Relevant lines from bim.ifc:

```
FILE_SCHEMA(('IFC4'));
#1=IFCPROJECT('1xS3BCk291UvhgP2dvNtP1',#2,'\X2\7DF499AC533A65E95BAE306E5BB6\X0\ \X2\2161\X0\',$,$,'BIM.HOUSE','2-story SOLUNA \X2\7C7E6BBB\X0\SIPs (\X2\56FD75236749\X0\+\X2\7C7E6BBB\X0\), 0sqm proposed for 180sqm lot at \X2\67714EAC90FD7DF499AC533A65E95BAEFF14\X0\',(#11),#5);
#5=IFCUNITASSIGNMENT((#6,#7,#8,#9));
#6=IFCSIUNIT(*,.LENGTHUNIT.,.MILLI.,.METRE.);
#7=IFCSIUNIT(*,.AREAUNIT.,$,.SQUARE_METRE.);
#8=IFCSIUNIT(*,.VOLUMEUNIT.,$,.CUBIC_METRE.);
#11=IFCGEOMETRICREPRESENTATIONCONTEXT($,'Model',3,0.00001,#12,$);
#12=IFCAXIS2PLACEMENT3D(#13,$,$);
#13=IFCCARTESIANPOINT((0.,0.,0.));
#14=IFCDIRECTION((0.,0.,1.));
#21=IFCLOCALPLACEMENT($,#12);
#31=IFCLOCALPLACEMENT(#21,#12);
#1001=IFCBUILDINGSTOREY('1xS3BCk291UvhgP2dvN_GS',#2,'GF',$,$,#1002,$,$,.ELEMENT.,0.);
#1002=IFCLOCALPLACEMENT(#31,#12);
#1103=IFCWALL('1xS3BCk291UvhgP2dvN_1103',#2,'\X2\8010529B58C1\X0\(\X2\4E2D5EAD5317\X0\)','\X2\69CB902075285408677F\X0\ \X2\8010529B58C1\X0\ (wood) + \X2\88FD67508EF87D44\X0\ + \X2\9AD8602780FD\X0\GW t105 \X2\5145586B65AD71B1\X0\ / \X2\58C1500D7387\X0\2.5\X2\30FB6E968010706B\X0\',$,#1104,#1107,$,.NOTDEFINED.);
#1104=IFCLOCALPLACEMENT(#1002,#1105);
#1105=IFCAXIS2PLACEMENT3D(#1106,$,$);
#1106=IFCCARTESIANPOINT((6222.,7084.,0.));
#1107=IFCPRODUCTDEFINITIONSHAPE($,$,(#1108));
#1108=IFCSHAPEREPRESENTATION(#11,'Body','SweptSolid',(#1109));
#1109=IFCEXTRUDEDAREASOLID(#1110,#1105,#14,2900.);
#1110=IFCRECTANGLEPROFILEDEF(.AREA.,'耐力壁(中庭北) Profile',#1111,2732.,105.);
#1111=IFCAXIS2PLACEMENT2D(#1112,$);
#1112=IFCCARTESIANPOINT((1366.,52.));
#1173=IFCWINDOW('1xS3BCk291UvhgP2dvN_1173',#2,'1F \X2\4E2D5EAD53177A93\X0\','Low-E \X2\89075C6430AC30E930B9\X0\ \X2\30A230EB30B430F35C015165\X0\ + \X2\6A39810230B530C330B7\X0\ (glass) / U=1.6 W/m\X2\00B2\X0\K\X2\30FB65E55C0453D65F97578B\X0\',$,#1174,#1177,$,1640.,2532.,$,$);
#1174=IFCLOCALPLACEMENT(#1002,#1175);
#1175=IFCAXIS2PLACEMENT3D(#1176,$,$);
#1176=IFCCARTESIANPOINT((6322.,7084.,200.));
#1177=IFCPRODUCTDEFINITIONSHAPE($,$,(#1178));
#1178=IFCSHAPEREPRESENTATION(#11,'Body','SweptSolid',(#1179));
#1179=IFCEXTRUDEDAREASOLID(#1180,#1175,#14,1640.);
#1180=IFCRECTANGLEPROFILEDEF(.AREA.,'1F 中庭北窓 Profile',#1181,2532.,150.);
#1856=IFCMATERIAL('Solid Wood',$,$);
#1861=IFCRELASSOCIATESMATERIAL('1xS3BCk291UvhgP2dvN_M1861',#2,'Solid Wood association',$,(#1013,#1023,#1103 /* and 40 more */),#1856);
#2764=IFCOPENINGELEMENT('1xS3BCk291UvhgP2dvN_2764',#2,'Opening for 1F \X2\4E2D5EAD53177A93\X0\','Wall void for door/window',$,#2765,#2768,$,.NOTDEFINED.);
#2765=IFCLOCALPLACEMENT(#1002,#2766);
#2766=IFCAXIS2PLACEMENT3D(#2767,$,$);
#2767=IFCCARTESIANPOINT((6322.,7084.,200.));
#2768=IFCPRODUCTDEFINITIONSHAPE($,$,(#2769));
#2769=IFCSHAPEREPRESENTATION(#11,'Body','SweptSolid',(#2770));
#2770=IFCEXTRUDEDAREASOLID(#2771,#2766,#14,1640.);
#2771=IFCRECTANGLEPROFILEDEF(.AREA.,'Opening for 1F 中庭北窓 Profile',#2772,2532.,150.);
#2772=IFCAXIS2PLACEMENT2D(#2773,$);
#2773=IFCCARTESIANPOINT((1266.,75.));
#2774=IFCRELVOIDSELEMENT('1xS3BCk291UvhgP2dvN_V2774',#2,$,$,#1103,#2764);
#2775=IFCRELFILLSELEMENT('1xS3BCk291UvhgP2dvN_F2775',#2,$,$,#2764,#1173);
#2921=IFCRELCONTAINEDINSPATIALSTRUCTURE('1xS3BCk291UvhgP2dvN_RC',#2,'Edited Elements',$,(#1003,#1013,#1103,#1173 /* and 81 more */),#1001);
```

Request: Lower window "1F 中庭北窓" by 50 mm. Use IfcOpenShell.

```python
import numpy as np
import ifcopenshell
import ifcopenshell.api.geometry
import ifcopenshell.util.placement
import ifcopenshell.util.unit

model = ifcopenshell.open("bim.ifc")
unit_scale = ifcopenshell.util.unit.calculate_unit_scale(model)

window = model.by_guid("1xS3BCk291UvhgP2dvN_1173")
opening = window.FillsVoids[0].RelatingOpeningElement
dz = -50.0

shift = np.array([0.0, 0.0, dz])
# The window is not placed relative to its opening, so move both.
for product in (opening, window):
    matrix = ifcopenshell.util.placement.get_local_placement(product.ObjectPlacement)
    matrix[:3, 3] += shift
    ifcopenshell.api.geometry.edit_object_placement(model, product=product, matrix=matrix, is_si=False)

print(f"moved by {dz * unit_scale:+.3f} m")

model.write("bim_edited.ifc")
```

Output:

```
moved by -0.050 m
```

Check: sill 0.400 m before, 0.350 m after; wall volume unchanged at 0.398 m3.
